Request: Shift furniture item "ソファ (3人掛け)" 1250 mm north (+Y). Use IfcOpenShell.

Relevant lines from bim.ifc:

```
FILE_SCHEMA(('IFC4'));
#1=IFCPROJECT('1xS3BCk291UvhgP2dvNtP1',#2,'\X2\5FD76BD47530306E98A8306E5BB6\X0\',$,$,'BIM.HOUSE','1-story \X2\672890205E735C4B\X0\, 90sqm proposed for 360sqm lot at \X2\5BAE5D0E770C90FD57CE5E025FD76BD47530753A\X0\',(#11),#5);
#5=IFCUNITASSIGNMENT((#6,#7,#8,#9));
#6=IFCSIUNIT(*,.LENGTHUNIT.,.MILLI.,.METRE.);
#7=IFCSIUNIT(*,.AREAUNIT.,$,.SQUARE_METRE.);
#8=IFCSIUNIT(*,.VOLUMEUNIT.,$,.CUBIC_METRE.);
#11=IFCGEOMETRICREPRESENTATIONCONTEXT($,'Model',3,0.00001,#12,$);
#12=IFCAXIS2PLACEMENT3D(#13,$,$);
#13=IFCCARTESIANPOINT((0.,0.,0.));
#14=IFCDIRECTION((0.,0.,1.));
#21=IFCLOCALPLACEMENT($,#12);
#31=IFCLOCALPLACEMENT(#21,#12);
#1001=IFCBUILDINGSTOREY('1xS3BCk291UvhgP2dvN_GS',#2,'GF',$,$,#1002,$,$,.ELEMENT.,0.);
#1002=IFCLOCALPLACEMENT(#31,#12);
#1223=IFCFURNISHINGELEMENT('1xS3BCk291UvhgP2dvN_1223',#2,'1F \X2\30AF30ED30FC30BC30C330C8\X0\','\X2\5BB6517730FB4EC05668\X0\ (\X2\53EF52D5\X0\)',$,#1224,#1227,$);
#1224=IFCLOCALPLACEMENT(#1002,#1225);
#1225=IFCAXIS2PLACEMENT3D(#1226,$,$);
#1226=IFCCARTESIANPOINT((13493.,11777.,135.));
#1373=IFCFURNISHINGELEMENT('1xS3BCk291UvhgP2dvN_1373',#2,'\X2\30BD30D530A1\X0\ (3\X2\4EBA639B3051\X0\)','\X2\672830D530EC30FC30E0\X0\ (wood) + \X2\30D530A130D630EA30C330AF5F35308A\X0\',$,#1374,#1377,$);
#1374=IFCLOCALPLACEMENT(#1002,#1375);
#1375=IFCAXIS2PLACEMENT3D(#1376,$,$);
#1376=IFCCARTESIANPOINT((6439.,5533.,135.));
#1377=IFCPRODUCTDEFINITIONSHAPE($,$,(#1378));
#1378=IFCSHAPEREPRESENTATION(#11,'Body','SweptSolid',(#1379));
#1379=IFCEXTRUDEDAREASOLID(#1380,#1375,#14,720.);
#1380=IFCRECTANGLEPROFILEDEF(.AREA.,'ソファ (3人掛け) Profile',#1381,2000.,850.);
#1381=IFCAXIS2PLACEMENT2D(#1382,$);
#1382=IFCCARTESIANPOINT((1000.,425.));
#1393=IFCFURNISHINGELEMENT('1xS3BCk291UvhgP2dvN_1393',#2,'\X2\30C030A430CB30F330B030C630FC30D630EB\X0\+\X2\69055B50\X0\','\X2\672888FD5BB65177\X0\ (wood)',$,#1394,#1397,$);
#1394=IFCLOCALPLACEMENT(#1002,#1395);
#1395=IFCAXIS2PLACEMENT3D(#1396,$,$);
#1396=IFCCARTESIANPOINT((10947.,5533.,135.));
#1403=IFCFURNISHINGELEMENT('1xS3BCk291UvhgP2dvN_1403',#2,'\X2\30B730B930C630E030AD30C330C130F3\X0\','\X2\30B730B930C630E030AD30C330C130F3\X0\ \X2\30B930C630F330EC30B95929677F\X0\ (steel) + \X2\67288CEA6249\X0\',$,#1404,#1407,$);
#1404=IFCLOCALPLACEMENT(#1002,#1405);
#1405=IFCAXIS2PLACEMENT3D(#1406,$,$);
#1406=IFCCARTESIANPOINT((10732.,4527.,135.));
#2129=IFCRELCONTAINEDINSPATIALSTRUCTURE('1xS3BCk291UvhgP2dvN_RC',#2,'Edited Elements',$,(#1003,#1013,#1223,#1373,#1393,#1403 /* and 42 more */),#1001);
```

```python
import ifcopenshell
import ifcopenshell.api.geometry
import ifcopenshell.util.placement

model = ifcopenshell.open("bim.ifc")

item = model.by_id(1373)
matrix = ifcopenshell.util.placement.get_local_placement(item.ObjectPlacement)
matrix[1, 3] += 1250.0
ifcopenshell.api.geometry.edit_object_placement(model, product=item, matrix=matrix, is_si=False)

print(ifcopenshell.util.placement.get_local_placement(item.ObjectPlacement).round(3) + 0.0)

model.write("bim_edited.ifc")
```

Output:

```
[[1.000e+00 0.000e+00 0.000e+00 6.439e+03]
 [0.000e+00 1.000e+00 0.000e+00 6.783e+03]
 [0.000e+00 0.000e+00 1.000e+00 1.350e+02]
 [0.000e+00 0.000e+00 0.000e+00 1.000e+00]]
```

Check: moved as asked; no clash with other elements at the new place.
